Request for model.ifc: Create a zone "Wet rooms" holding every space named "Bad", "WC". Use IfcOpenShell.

First a look at what the model holds.

```python
import ifcopenshell

model = ifcopenshell.open("model.ifc")
print(model.schema)
seen = {}
for space in model.by_type("IfcSpace"):
    seen[space.LongName] = seen.get(space.LongName, 0) + 1
for name, count in sorted(seen.items(), key=str):
    print(count, "x", name)
print("zones:", [z.Name for z in model.by_type("IfcZone")][:20])
```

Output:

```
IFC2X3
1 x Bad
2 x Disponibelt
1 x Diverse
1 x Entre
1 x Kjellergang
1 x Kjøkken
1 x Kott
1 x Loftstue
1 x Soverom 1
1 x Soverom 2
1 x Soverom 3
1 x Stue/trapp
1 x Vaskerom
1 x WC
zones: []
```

```python
import ifcopenshell
import ifcopenshell.api.group
import ifcopenshell.api.root

model = ifcopenshell.open("model.ifc")

names = {"Bad", "WC"}
spaces = [s for s in model.by_type("IfcSpace") if s.LongName in names]

zone = ifcopenshell.api.root.create_entity(model, ifc_class="IfcZone", name="Wet rooms")
ifcopenshell.api.group.assign_group(model, products=spaces, group=zone)
print(len(spaces), "spaces in", zone.Name)

model.write("model-out.ifc")
```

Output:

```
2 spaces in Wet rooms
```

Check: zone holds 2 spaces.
